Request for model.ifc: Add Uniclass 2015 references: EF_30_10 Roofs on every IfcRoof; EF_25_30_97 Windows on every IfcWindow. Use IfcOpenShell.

First a look at what the model holds.

```python
import ifcopenshell

model = ifcopenshell.open("model.ifc")
print(model.schema)
print("classifications:", [c.Name for c in model.by_type("IfcClassification")])
for ifc_class in ("IfcDoor", "IfcRoof", "IfcStair", "IfcWall", "IfcWindow"):
    print(ifc_class, len(model.by_type(ifc_class)))
```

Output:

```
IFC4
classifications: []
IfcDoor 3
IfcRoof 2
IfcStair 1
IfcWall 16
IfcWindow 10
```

```python
import ifcopenshell
import ifcopenshell.api.classification

model = ifcopenshell.open("model.ifc")

system = ifcopenshell.api.classification.add_classification(model, classification="Uniclass 2015")

codes = {
    "IfcRoof": ("EF_30_10", "Roofs"),
    "IfcWindow": ("EF_25_30_97", "Windows"),
}
for ifc_class, (code, name) in codes.items():
    products = model.by_type(ifc_class)
    ifcopenshell.api.classification.add_reference(
        model, products=products, classification=system, identification=code, name=name
    )
    print(code, len(products))

model.write("model_rev.ifc")
```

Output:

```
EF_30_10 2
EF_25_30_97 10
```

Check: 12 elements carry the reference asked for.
